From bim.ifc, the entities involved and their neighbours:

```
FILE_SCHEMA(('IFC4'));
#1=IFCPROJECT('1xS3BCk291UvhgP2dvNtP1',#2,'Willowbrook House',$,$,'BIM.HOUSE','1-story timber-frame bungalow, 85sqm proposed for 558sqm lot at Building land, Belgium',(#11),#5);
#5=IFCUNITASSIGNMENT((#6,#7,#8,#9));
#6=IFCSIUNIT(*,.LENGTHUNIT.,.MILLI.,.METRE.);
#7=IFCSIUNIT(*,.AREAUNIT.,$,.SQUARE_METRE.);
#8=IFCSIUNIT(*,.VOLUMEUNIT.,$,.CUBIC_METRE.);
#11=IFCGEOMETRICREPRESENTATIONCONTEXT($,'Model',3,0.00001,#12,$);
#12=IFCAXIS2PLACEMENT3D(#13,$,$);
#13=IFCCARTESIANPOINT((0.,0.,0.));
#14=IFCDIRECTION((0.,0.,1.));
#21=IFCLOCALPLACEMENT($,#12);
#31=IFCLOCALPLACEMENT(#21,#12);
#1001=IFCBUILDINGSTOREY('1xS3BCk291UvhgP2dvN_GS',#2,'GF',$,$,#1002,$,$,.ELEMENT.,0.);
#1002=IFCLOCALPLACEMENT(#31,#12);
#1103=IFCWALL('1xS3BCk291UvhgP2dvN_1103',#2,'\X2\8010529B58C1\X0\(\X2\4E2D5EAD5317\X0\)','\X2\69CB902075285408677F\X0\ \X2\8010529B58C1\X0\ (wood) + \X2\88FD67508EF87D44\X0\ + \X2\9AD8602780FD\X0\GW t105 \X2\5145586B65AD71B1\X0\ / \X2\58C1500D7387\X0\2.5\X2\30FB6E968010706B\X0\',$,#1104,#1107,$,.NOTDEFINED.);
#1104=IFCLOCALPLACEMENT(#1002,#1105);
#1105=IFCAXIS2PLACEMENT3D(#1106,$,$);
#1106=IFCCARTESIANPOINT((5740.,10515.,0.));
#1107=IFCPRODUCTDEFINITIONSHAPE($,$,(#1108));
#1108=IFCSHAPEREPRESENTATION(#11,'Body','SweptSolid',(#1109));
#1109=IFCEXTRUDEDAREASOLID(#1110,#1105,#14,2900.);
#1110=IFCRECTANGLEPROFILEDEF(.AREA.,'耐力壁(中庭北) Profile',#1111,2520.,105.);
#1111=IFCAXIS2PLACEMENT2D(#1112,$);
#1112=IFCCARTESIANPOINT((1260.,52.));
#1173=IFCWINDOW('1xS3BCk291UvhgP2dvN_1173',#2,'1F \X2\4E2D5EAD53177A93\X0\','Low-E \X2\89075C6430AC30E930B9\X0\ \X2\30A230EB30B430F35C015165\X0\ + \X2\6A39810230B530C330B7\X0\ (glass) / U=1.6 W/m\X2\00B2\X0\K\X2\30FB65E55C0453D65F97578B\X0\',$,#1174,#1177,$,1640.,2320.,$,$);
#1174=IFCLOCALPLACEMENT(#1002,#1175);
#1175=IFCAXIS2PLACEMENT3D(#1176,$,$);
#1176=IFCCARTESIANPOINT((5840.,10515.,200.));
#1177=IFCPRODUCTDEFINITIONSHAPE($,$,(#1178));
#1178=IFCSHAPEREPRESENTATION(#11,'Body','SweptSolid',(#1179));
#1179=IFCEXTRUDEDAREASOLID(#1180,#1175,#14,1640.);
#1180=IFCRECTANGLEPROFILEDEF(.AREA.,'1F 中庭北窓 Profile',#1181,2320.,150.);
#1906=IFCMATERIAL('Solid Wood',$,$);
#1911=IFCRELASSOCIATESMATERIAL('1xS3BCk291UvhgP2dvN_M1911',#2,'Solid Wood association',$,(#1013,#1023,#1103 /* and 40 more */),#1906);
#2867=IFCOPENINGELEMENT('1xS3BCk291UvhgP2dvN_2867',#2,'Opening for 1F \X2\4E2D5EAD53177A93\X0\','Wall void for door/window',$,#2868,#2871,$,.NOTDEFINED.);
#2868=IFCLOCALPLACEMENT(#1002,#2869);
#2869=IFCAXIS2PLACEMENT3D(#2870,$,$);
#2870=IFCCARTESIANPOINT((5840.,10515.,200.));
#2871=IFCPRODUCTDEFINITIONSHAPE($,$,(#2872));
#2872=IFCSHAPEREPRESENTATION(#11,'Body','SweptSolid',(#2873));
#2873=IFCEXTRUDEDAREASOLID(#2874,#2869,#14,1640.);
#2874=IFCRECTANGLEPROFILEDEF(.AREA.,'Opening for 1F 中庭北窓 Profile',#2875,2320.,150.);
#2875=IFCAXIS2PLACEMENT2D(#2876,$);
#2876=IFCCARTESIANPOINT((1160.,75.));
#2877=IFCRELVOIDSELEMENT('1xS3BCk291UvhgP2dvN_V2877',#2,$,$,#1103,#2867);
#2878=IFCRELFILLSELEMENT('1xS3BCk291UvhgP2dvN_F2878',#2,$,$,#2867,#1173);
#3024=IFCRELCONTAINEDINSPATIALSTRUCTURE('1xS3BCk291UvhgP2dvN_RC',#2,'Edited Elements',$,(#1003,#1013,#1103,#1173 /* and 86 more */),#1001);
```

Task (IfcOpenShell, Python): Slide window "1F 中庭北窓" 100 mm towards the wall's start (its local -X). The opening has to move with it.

```python
import ifcopenshell
import ifcopenshell.api.geometry
import ifcopenshell.util.placement

model = ifcopenshell.open("bim.ifc")

window = model.by_id(1173)
opening = window.FillsVoids[0].RelatingOpeningElement
wall = opening.VoidsElements[0].RelatingBuildingElement

wall_matrix = ifcopenshell.util.placement.get_local_placement(wall.ObjectPlacement)
shift = wall_matrix[:3, 0] * -100.0
before = ifcopenshell.util.placement.get_local_placement(window.ObjectPlacement)[:3, 3].copy()

# The window is not placed relative to its opening, so move both.
for product in (opening, window):
    matrix = ifcopenshell.util.placement.get_local_placement(product.ObjectPlacement)
    matrix[:3, 3] += shift
    ifcopenshell.api.geometry.edit_object_placement(model, product=product, matrix=matrix, is_si=False)

after = ifcopenshell.util.placement.get_local_placement(window.ObjectPlacement)[:3, 3]
print("window moved by", (after - before).round(3) + 0.0)

model.write("bim_v2.ifc")
```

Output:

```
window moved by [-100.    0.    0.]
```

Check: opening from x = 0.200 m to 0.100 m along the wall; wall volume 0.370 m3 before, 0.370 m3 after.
